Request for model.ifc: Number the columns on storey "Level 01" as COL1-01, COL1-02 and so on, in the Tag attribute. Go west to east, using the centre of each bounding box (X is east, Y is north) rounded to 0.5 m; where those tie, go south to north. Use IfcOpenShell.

First a look at what the model holds.

```python
import ifcopenshell
import ifcopenshell.util.element
import ifcopenshell.util.placement

model = ifcopenshell.open("model.ifc")
print(model.schema)
storey = next(s for s in model.by_type("IfcBuildingStorey") if s.Name == "Level 01")
columns = [e for e in ifcopenshell.util.element.get_decomposition(storey) if e.is_a("IfcColumn")]
for e in sorted(columns, key=lambda e: e.id()):
    origin = ifcopenshell.util.placement.get_local_placement(e.ObjectPlacement)[:3, 3]
    print(e.id(), e.Tag, e.Name, origin.round(2) + 0.0, sep=" | ")
```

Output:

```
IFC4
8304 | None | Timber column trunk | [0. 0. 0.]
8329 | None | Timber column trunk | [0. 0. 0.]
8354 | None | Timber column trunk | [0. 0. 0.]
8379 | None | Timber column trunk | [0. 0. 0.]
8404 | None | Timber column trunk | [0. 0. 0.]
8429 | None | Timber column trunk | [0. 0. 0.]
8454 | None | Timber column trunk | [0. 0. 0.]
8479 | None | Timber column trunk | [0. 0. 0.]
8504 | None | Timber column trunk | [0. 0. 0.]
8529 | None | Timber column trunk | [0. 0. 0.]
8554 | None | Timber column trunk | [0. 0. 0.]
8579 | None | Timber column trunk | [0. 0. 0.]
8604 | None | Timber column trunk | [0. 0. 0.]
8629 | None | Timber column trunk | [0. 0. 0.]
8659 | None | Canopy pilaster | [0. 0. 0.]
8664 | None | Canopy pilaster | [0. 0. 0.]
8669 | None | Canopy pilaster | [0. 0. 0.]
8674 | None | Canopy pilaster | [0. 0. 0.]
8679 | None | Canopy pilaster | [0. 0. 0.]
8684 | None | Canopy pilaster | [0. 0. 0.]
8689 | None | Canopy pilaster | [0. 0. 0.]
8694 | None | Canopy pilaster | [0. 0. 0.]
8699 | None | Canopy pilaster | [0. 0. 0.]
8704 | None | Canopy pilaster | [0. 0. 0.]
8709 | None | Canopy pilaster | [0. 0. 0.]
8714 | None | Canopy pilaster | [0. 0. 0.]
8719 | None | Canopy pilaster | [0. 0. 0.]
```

```python
import ifcopenshell
import ifcopenshell.geom
import ifcopenshell.util.element
import ifcopenshell.util.shape

model = ifcopenshell.open("model.ifc")
settings = ifcopenshell.geom.settings()
settings.set("use-world-coords", True)


def centre(element):
    shape = ifcopenshell.geom.create_shape(settings, element)
    return ifcopenshell.util.shape.get_bbox_centroid(shape.geometry)


storey = next(s for s in model.by_type("IfcBuildingStorey") if s.Name == "Level 01")
columns = [e for e in ifcopenshell.util.element.get_decomposition(storey) if e.is_a("IfcColumn")]

# Insertion points can sit at a corner or the storey origin, so sort by the geometry (in metres).
centres = {e: centre(e) for e in columns}
columns.sort(key=lambda e: (round(centres[e][0] / 0.5), centres[e][1]))

for i, e in enumerate(columns, start=1):
    number = f"COL1-{i:02d}"
    e.Tag = number
    print(e.id(), number)

model.write("model-out.ifc")
```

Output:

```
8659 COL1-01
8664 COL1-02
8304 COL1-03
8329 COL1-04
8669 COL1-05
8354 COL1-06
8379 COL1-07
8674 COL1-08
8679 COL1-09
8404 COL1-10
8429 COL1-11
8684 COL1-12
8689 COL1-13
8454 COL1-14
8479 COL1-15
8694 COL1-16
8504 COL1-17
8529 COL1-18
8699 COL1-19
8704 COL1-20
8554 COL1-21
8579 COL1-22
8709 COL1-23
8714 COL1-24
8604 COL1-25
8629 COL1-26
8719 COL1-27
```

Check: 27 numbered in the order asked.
